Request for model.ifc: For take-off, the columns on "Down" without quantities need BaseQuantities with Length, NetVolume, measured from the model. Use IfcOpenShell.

First a look at what the model holds.

```python
import ifcopenshell
import ifcopenshell.util.element
import ifcopenshell.util.unit

model = ifcopenshell.open("model.ifc")
print(model.schema)
for unit_type in ("LENGTHUNIT", "AREAUNIT", "VOLUMEUNIT"):
    print(unit_type, ifcopenshell.util.unit.calculate_unit_scale(model, unit_type))
storey = next(s for s in model.by_type("IfcBuildingStorey") if s.Name == "Down")
columns = [e for e in ifcopenshell.util.element.get_decomposition(storey) if e.is_a("IfcColumn")]
for e in sorted(columns, key=lambda e: e.id()):
    print(e.id(), e.is_a(), e.Name, list(ifcopenshell.util.element.get_psets(e, qtos_only=True)), sep=" | ")
```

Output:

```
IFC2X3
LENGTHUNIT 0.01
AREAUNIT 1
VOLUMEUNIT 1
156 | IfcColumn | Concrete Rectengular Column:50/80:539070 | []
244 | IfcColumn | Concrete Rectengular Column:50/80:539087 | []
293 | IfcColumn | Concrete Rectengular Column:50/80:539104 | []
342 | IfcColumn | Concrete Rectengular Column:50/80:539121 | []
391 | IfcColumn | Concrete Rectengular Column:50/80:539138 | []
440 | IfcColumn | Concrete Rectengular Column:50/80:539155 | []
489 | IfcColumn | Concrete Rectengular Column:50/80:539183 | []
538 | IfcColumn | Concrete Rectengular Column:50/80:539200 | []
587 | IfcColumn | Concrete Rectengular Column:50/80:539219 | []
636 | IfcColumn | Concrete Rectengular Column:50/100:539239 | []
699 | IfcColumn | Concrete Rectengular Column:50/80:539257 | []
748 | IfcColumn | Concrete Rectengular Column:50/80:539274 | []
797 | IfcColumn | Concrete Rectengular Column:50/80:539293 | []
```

```python
import ifcopenshell
import ifcopenshell.api.pset
import ifcopenshell.geom
import ifcopenshell.util.element
import ifcopenshell.util.shape
import ifcopenshell.util.unit

model = ifcopenshell.open("model.ifc")
unit_scale = ifcopenshell.util.unit.calculate_unit_scale(model)
volume_scale = ifcopenshell.util.unit.calculate_unit_scale(model, "VOLUMEUNIT")
settings = ifcopenshell.geom.settings()

storey = next(s for s in model.by_type("IfcBuildingStorey") if s.Name == "Down")
columns = [e for e in ifcopenshell.util.element.get_decomposition(storey) if e.is_a("IfcColumn")]

for e in sorted(columns, key=lambda e: e.id()):
    if ifcopenshell.util.element.get_psets(e, qtos_only=True, should_inherit=False):
        continue
    # Geometry comes back in metres, in the element's own axes.
    shape = ifcopenshell.geom.create_shape(settings, e)
    values = {
        "Length": ifcopenshell.util.shape.get_z(shape.geometry) / unit_scale,
        "NetVolume": ifcopenshell.util.shape.get_volume(shape.geometry) / volume_scale,
    }
    qto = ifcopenshell.api.pset.add_qto(model, product=e, name="BaseQuantities")
    ifcopenshell.api.pset.edit_qto(model, qto=qto, properties=values)
    print(e.id(), {k: round(v, 3) for k, v in values.items()})

model.write("model_edited.ifc")
```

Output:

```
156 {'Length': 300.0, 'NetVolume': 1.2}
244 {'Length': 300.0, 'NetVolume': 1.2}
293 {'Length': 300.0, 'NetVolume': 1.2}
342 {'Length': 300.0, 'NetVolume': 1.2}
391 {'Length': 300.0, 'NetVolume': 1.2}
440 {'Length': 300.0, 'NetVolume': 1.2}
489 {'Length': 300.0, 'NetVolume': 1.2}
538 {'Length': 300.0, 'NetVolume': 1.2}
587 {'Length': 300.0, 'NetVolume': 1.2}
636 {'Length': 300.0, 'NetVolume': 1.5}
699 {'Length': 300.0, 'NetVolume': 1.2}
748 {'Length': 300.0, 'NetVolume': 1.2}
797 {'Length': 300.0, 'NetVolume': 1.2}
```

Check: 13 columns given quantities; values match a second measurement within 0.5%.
